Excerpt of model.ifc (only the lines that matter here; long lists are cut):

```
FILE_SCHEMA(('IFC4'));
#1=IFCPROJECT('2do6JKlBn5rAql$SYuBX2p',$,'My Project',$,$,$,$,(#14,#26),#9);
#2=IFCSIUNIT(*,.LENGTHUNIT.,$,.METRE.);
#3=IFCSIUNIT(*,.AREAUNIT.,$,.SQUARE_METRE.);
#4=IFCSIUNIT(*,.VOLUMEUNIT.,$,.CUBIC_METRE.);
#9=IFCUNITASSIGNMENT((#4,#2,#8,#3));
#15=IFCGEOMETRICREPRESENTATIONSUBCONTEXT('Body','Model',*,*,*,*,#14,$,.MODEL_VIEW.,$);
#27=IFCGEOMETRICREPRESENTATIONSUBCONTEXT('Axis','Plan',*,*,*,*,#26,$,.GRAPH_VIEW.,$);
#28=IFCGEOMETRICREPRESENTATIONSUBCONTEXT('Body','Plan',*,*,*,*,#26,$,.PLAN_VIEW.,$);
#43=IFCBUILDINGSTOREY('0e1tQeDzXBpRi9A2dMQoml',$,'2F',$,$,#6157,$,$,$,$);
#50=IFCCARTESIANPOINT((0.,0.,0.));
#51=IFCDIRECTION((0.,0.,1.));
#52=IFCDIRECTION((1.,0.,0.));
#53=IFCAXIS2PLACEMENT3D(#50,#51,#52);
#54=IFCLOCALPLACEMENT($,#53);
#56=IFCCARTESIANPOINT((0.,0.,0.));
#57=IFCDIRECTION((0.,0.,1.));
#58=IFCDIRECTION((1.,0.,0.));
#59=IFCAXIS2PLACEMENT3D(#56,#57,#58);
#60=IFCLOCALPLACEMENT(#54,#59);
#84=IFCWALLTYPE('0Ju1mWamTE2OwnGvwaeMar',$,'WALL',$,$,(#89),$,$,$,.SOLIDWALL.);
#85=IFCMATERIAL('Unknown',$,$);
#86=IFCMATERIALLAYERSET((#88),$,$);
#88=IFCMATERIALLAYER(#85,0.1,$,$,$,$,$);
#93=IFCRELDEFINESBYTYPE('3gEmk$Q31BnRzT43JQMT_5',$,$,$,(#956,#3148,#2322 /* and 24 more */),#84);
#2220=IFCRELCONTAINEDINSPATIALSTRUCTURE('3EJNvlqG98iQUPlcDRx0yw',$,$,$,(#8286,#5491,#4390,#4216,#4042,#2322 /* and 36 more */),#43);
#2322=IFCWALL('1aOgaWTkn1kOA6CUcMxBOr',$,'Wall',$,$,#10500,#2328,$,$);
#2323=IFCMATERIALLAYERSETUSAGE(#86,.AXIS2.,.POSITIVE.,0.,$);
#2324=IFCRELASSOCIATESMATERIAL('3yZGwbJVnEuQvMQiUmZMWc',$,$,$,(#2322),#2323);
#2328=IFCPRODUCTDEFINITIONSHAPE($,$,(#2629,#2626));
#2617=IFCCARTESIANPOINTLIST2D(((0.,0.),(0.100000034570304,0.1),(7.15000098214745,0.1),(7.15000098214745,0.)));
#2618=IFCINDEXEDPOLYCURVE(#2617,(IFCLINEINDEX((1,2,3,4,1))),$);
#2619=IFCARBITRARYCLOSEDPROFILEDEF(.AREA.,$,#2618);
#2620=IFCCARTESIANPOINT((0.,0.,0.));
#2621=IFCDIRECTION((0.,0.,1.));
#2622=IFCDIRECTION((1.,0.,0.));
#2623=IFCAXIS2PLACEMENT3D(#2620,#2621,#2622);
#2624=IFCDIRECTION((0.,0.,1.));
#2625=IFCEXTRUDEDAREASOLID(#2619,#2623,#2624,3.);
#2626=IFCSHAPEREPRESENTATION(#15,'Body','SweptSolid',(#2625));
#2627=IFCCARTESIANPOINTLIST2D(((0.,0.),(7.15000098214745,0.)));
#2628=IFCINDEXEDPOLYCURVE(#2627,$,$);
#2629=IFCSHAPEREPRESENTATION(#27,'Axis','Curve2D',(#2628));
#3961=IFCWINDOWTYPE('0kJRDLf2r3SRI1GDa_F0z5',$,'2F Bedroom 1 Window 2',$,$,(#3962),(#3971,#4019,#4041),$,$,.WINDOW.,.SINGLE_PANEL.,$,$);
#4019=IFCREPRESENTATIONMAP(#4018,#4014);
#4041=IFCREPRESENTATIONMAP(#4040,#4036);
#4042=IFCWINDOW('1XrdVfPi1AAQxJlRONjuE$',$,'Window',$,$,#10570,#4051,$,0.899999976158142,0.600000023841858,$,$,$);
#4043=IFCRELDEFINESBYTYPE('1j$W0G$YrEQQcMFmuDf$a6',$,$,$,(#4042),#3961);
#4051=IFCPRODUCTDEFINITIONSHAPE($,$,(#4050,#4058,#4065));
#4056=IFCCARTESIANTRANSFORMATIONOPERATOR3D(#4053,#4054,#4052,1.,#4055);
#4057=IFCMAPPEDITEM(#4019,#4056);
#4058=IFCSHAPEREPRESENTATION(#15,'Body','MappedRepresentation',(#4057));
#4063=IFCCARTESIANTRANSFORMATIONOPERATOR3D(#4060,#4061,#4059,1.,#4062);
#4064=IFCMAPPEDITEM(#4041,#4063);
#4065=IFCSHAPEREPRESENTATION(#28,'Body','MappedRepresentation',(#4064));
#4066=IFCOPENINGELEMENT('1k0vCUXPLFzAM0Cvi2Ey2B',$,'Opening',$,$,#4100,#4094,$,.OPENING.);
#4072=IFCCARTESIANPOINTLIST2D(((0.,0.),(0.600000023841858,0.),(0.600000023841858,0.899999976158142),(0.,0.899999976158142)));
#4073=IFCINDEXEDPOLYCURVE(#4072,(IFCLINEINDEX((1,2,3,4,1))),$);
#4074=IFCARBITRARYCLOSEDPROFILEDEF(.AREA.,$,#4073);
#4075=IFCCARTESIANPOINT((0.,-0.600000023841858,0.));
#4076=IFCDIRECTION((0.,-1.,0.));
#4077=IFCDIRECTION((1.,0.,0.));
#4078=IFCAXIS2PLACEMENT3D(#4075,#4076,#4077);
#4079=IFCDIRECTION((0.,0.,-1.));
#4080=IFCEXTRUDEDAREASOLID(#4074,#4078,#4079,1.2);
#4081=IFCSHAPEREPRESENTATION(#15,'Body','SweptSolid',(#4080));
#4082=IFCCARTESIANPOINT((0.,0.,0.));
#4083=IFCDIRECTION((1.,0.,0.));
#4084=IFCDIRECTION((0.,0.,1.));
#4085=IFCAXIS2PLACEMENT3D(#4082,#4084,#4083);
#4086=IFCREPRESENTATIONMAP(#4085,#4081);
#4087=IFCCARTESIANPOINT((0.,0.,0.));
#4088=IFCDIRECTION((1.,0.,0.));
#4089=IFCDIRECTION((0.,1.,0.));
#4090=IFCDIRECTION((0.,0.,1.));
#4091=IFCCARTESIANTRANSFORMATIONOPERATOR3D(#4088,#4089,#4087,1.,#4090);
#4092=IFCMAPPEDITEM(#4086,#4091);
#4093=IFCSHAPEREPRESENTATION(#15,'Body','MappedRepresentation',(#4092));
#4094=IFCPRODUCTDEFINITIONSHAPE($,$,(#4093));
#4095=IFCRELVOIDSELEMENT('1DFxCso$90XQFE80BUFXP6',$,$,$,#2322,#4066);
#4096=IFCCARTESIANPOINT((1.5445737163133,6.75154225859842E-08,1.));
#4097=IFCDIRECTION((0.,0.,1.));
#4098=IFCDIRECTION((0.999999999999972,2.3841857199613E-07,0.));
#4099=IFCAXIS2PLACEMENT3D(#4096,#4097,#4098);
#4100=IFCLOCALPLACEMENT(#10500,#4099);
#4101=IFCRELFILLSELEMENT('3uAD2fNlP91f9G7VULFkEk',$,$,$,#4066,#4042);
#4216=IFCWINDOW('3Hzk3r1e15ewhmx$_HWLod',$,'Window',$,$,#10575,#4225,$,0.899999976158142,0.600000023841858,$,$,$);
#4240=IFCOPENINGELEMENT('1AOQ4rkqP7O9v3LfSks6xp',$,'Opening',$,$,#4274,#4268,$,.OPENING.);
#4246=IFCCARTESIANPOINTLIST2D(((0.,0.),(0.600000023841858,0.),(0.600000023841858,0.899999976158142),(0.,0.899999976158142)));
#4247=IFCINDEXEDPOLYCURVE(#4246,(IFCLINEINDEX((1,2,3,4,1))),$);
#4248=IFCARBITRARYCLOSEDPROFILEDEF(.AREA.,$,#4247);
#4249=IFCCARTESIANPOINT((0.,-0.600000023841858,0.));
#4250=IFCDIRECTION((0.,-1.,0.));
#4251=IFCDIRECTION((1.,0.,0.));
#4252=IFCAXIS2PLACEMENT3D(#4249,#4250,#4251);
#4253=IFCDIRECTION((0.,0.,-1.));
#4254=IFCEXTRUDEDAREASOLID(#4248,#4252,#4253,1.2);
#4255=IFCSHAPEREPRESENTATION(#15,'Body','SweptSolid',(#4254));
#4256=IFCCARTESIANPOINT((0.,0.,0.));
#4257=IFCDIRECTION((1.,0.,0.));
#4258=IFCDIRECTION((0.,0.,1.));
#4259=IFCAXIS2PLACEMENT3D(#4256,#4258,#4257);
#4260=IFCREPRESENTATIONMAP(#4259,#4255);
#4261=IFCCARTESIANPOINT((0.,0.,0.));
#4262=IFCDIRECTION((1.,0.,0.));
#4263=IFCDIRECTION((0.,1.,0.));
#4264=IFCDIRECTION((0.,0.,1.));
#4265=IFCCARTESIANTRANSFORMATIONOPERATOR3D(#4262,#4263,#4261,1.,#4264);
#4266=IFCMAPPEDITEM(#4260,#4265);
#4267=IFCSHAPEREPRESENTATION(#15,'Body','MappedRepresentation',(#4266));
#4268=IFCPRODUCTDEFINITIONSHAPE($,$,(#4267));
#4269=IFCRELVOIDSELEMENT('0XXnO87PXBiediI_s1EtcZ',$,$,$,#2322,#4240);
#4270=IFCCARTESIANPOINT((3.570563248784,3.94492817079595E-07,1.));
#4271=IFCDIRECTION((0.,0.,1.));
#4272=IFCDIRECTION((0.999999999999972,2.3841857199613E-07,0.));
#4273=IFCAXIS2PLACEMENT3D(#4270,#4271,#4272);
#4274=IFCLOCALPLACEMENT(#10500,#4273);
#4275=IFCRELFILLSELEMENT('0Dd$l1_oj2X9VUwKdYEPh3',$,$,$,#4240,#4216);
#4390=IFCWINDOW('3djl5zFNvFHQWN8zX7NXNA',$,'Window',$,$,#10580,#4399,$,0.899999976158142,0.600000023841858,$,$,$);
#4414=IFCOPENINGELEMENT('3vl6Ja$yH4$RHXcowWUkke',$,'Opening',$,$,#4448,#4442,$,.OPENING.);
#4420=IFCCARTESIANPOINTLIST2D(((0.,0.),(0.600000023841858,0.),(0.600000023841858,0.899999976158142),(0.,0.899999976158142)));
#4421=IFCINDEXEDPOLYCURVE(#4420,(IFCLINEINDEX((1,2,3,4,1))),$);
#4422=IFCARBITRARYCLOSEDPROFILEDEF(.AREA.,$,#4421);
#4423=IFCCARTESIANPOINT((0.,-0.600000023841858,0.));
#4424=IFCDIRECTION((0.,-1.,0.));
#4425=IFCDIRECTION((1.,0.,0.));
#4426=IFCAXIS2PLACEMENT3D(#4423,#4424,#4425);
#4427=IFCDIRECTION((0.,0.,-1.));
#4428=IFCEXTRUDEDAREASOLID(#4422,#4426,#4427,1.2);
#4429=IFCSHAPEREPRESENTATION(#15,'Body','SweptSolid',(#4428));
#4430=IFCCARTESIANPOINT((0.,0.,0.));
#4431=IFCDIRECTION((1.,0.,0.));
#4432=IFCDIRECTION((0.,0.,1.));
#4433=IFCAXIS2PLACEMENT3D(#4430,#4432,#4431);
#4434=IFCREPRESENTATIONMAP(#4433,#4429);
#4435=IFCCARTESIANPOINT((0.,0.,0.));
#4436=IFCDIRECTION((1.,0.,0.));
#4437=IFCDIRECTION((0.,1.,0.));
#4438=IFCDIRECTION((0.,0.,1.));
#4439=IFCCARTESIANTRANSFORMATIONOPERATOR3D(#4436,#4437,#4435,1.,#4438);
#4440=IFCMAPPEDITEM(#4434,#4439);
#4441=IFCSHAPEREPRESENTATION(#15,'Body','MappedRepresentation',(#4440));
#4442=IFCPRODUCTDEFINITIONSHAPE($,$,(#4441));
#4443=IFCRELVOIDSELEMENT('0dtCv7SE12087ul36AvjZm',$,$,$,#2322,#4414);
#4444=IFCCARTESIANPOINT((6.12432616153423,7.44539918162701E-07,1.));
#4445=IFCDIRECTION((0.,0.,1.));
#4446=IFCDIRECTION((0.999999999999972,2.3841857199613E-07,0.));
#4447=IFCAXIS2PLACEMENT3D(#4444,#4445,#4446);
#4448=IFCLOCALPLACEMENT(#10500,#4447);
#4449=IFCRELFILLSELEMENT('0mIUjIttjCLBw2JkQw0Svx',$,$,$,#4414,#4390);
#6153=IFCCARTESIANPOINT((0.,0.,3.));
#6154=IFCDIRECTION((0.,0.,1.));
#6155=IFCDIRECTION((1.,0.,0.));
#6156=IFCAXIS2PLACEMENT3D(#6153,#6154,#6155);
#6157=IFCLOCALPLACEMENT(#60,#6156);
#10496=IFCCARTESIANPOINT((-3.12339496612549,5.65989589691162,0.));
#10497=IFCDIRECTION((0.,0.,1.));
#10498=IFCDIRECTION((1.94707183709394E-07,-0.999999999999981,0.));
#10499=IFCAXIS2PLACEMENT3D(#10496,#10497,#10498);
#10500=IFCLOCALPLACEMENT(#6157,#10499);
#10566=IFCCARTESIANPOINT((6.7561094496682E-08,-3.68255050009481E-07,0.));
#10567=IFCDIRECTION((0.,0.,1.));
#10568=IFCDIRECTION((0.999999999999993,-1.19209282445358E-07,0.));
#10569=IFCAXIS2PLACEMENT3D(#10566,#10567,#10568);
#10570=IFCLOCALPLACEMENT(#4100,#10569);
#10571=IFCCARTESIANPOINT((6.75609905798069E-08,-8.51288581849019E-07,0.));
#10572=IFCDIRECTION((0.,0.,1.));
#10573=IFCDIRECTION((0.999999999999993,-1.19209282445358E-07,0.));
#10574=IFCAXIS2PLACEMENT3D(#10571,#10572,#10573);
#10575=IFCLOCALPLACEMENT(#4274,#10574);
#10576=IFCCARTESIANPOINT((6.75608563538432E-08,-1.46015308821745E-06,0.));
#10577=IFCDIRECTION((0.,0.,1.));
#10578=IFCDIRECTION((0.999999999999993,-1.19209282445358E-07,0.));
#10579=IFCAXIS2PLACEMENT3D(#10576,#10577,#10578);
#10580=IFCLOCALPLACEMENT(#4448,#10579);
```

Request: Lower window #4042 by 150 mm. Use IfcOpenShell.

```python
import numpy as np
import ifcopenshell
import ifcopenshell.api.geometry
import ifcopenshell.util.placement
import ifcopenshell.util.unit

model = ifcopenshell.open("model.ifc")
unit_scale = ifcopenshell.util.unit.calculate_unit_scale(model)

window = model.by_guid("1XrdVfPi1AAQxJlRONjuE$")
opening = window.FillsVoids[0].RelatingOpeningElement
dz = -0.15

shift = np.array([0.0, 0.0, dz])
# The window is placed relative to its opening, so it follows when the opening moves.
matrix = ifcopenshell.util.placement.get_local_placement(opening.ObjectPlacement)
matrix[:3, 3] += shift
ifcopenshell.api.geometry.edit_object_placement(
    model, product=opening, matrix=matrix, is_si=False, should_transform_children=True
)

print(f"moved by {dz * unit_scale:+.3f} m")

model.write("model_rev.ifc")
```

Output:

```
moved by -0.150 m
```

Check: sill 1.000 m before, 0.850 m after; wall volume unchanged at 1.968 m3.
